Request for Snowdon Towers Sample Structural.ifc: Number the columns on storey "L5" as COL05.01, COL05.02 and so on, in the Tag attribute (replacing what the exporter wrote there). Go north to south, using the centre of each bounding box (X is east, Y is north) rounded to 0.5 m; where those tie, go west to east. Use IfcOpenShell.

First a look at what the model holds.

```python
import ifcopenshell
import ifcopenshell.util.element
import ifcopenshell.util.placement

model = ifcopenshell.open("Snowdon Towers Sample Structural.ifc")
print(model.schema)
storey = next(s for s in model.by_type("IfcBuildingStorey") if s.Name == "L5")
columns = [e for e in ifcopenshell.util.element.get_decomposition(storey) if e.is_a("IfcColumn")]
for e in sorted(columns, key=lambda e: e.id()):
    origin = ifcopenshell.util.placement.get_local_placement(e.ObjectPlacement)[:3, 3]
    print(e.id(), e.Tag, e.Name, origin.round(2) + 0.0, sep=" | ")
```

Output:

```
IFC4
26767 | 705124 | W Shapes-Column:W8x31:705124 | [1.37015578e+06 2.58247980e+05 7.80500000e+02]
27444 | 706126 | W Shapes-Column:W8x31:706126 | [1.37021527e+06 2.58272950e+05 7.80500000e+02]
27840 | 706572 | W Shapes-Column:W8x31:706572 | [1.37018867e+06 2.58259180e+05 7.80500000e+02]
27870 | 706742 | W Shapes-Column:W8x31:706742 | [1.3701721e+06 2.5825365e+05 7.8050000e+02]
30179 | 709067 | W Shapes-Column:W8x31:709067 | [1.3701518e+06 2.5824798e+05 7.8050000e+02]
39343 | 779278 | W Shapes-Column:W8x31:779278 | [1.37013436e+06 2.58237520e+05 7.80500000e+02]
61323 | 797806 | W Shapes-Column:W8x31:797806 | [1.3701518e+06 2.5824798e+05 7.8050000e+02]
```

```python
import ifcopenshell
import ifcopenshell.geom
import ifcopenshell.util.element
import ifcopenshell.util.shape

model = ifcopenshell.open("Snowdon Towers Sample Structural.ifc")
settings = ifcopenshell.geom.settings()
settings.set("use-world-coords", True)


def centre(element):
    shape = ifcopenshell.geom.create_shape(settings, element)
    return ifcopenshell.util.shape.get_bbox_centroid(shape.geometry)


storey = next(s for s in model.by_type("IfcBuildingStorey") if s.Name == "L5")
columns = [e for e in ifcopenshell.util.element.get_decomposition(storey) if e.is_a("IfcColumn")]

# Insertion points can sit at a corner or the storey origin, so sort by the geometry (in metres).
centres = {e: centre(e) for e in columns}
columns.sort(key=lambda e: (-round(centres[e][1] / 0.5), centres[e][0]))

for i, e in enumerate(columns, start=1):
    number = f"COL05.{i:02d}"
    e.Tag = number
    print(e.id(), number)

model.write("Snowdon Towers Sample Structural-out.ifc")
```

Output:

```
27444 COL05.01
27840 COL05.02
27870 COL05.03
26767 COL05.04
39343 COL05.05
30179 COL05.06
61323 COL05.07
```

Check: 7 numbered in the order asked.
